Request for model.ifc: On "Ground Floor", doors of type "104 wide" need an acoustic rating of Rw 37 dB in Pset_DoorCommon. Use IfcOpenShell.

First a look at what the model holds.

```python
import ifcopenshell
import ifcopenshell.util.element

model = ifcopenshell.open("model.ifc")
print(model.schema)
storey = next(s for s in model.by_type("IfcBuildingStorey") if s.Name == "Ground Floor")
doors = [e for e in ifcopenshell.util.element.get_decomposition(storey) if e.is_a("IfcDoor")]
seen = {}
for e in doors:
    element_type = ifcopenshell.util.element.get_type(e)
    key = (element_type.Name if element_type != e and element_type else None, ifcopenshell.util.element.get_pset(e, "Pset_DoorCommon", "AcousticRating"))
    seen[key] = seen.get(key, 0) + 1
for (name, value), count in sorted(seen.items(), key=str):
    print(count, "x", name, "|", value)
```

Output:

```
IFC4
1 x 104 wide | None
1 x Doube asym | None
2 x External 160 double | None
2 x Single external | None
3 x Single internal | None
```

```python
import ifcopenshell
import ifcopenshell.api.pset
import ifcopenshell.util.element

model = ifcopenshell.open("model.ifc")

storey = next(s for s in model.by_type("IfcBuildingStorey") if s.Name == "Ground Floor")
doors = [e for e in ifcopenshell.util.element.get_decomposition(storey) if e.is_a("IfcDoor")]

count = 0
for e in doors:
    element_type = ifcopenshell.util.element.get_type(e)
    if element_type in (None, e) or element_type.Name != "104 wide":
        continue
    # add_pset returns the element's existing set when there is one.
    pset = ifcopenshell.api.pset.add_pset(model, product=e, name="Pset_DoorCommon")
    ifcopenshell.api.pset.edit_pset(model, pset=pset, properties={"AcousticRating": "Rw 37 dB"})
    count += 1

print(count, "doors updated")

model.write("model_edited.ifc")
```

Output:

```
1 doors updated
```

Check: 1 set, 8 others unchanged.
